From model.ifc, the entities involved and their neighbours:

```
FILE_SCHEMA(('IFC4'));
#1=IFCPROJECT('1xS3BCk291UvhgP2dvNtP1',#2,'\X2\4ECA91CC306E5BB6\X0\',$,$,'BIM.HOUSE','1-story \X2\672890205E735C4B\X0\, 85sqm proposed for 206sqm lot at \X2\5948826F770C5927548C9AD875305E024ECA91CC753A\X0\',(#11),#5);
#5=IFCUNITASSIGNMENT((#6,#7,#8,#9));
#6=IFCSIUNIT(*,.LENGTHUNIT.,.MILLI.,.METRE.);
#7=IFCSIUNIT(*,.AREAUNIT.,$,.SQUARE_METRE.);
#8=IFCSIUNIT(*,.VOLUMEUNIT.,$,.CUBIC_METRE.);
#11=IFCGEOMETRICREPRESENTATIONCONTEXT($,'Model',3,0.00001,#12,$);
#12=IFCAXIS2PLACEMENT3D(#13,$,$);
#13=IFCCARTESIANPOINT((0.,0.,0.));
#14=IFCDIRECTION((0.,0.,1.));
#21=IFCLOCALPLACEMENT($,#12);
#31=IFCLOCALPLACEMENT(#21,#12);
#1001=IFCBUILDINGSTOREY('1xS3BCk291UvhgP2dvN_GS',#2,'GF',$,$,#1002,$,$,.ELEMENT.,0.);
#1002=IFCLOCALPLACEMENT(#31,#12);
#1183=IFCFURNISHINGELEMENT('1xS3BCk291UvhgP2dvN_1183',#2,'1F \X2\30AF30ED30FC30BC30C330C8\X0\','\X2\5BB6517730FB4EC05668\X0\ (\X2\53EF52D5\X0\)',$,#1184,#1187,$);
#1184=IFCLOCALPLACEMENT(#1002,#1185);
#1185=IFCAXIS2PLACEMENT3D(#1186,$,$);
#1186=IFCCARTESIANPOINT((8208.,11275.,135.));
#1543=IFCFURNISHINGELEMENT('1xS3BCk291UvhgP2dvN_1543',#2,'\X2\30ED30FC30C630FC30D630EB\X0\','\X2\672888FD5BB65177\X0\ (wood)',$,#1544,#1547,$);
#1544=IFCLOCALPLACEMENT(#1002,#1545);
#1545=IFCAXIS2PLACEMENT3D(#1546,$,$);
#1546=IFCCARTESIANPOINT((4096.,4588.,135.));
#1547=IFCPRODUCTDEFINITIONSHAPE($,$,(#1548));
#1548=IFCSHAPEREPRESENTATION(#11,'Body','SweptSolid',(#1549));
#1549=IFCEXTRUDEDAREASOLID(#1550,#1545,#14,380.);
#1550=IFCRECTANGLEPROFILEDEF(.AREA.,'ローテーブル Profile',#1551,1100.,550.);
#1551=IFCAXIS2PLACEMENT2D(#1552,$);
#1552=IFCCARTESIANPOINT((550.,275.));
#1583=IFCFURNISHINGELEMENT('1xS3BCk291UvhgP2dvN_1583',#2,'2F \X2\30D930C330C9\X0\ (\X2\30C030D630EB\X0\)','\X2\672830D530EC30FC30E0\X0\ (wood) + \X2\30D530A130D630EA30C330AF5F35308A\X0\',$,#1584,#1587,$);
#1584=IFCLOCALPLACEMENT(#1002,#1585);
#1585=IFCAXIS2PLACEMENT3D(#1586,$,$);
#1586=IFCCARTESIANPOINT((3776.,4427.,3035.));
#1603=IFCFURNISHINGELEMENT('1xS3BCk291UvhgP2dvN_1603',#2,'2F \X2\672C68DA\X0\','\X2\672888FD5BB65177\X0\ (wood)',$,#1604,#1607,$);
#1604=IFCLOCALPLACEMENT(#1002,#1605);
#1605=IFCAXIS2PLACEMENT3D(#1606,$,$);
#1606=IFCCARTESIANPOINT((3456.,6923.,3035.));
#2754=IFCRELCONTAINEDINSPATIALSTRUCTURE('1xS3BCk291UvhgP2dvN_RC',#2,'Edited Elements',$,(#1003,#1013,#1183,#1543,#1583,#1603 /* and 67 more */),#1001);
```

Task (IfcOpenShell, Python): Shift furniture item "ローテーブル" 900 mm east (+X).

```python
import ifcopenshell
import ifcopenshell.api.geometry
import ifcopenshell.util.placement
import ifcopenshell.util.unit

model = ifcopenshell.open("model.ifc")
unit_scale = ifcopenshell.util.unit.calculate_unit_scale(model)

item = model.by_id(1543)
matrix = ifcopenshell.util.placement.get_local_placement(item.ObjectPlacement)
matrix[0, 3] += 0.9 / unit_scale
ifcopenshell.api.geometry.edit_object_placement(model, product=item, matrix=matrix, is_si=False)

print(ifcopenshell.util.placement.get_local_placement(item.ObjectPlacement).round(3) + 0.0)

model.write("model-out.ifc")
```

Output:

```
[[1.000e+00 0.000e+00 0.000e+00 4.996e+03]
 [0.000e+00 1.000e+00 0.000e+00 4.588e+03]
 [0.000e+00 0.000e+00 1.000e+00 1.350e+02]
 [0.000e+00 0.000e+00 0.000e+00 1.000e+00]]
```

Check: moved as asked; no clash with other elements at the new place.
